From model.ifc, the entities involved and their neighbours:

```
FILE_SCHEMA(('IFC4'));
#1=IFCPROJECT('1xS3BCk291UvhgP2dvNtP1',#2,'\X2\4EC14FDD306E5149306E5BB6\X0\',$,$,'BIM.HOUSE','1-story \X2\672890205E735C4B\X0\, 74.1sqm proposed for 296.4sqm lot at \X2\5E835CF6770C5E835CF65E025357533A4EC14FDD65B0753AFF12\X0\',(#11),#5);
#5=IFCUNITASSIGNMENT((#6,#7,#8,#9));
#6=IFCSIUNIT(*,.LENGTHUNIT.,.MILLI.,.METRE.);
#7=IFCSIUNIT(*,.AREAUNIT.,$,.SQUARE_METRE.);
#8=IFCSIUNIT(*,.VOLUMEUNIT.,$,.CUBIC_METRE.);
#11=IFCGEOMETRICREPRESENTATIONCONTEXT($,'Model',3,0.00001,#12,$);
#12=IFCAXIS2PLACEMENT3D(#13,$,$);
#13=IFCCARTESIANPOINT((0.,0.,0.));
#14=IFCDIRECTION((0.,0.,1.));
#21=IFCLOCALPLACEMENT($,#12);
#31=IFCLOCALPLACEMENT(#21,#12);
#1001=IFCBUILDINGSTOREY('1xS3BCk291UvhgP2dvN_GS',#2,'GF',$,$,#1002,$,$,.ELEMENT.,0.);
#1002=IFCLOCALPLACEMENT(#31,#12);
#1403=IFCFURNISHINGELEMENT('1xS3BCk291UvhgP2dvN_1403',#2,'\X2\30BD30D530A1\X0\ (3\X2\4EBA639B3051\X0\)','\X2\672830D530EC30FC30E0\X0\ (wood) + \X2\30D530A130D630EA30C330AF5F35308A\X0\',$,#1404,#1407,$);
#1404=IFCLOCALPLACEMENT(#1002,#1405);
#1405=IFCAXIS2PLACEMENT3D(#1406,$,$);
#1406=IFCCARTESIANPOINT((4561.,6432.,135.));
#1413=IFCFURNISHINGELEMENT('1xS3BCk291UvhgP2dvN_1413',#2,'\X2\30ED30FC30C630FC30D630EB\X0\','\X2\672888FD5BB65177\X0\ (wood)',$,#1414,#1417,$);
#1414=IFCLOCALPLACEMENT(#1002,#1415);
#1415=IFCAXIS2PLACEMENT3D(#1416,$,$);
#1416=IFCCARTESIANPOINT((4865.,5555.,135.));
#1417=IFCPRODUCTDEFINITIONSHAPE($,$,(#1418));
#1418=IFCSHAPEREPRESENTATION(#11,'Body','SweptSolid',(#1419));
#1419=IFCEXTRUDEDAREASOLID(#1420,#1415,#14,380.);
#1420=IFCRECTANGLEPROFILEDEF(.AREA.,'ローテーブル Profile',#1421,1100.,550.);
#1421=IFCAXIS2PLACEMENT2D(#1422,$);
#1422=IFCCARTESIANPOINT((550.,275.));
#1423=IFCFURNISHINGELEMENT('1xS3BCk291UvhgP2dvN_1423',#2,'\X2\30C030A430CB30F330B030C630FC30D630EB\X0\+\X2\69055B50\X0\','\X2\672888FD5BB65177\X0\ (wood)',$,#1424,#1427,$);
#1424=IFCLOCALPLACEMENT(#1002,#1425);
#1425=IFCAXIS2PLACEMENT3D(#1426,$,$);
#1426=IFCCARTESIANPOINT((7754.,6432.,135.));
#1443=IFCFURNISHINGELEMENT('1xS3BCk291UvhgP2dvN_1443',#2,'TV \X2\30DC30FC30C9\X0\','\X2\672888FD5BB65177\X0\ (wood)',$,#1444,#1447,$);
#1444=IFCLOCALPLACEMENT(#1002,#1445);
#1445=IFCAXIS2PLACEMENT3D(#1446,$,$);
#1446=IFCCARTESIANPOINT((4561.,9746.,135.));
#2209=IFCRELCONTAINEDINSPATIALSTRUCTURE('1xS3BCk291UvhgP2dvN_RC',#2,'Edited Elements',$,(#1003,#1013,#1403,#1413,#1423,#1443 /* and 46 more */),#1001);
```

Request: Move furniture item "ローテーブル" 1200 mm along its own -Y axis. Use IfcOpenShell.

```python
import ifcopenshell
import ifcopenshell.api.geometry
import ifcopenshell.util.placement

model = ifcopenshell.open("model.ifc")

item = model.by_id(1413)
matrix = ifcopenshell.util.placement.get_local_placement(item.ObjectPlacement)
matrix[:3, 3] -= matrix[:3, 1] * 1200.0
ifcopenshell.api.geometry.edit_object_placement(model, product=item, matrix=matrix, is_si=False)

print(ifcopenshell.util.placement.get_local_placement(item.ObjectPlacement).round(3) + 0.0)

model.write("model_rev.ifc")
```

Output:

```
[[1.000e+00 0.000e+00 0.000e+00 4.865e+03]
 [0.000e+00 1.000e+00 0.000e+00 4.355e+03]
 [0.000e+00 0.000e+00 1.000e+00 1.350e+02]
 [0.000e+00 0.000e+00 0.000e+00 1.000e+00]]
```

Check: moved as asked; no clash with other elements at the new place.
